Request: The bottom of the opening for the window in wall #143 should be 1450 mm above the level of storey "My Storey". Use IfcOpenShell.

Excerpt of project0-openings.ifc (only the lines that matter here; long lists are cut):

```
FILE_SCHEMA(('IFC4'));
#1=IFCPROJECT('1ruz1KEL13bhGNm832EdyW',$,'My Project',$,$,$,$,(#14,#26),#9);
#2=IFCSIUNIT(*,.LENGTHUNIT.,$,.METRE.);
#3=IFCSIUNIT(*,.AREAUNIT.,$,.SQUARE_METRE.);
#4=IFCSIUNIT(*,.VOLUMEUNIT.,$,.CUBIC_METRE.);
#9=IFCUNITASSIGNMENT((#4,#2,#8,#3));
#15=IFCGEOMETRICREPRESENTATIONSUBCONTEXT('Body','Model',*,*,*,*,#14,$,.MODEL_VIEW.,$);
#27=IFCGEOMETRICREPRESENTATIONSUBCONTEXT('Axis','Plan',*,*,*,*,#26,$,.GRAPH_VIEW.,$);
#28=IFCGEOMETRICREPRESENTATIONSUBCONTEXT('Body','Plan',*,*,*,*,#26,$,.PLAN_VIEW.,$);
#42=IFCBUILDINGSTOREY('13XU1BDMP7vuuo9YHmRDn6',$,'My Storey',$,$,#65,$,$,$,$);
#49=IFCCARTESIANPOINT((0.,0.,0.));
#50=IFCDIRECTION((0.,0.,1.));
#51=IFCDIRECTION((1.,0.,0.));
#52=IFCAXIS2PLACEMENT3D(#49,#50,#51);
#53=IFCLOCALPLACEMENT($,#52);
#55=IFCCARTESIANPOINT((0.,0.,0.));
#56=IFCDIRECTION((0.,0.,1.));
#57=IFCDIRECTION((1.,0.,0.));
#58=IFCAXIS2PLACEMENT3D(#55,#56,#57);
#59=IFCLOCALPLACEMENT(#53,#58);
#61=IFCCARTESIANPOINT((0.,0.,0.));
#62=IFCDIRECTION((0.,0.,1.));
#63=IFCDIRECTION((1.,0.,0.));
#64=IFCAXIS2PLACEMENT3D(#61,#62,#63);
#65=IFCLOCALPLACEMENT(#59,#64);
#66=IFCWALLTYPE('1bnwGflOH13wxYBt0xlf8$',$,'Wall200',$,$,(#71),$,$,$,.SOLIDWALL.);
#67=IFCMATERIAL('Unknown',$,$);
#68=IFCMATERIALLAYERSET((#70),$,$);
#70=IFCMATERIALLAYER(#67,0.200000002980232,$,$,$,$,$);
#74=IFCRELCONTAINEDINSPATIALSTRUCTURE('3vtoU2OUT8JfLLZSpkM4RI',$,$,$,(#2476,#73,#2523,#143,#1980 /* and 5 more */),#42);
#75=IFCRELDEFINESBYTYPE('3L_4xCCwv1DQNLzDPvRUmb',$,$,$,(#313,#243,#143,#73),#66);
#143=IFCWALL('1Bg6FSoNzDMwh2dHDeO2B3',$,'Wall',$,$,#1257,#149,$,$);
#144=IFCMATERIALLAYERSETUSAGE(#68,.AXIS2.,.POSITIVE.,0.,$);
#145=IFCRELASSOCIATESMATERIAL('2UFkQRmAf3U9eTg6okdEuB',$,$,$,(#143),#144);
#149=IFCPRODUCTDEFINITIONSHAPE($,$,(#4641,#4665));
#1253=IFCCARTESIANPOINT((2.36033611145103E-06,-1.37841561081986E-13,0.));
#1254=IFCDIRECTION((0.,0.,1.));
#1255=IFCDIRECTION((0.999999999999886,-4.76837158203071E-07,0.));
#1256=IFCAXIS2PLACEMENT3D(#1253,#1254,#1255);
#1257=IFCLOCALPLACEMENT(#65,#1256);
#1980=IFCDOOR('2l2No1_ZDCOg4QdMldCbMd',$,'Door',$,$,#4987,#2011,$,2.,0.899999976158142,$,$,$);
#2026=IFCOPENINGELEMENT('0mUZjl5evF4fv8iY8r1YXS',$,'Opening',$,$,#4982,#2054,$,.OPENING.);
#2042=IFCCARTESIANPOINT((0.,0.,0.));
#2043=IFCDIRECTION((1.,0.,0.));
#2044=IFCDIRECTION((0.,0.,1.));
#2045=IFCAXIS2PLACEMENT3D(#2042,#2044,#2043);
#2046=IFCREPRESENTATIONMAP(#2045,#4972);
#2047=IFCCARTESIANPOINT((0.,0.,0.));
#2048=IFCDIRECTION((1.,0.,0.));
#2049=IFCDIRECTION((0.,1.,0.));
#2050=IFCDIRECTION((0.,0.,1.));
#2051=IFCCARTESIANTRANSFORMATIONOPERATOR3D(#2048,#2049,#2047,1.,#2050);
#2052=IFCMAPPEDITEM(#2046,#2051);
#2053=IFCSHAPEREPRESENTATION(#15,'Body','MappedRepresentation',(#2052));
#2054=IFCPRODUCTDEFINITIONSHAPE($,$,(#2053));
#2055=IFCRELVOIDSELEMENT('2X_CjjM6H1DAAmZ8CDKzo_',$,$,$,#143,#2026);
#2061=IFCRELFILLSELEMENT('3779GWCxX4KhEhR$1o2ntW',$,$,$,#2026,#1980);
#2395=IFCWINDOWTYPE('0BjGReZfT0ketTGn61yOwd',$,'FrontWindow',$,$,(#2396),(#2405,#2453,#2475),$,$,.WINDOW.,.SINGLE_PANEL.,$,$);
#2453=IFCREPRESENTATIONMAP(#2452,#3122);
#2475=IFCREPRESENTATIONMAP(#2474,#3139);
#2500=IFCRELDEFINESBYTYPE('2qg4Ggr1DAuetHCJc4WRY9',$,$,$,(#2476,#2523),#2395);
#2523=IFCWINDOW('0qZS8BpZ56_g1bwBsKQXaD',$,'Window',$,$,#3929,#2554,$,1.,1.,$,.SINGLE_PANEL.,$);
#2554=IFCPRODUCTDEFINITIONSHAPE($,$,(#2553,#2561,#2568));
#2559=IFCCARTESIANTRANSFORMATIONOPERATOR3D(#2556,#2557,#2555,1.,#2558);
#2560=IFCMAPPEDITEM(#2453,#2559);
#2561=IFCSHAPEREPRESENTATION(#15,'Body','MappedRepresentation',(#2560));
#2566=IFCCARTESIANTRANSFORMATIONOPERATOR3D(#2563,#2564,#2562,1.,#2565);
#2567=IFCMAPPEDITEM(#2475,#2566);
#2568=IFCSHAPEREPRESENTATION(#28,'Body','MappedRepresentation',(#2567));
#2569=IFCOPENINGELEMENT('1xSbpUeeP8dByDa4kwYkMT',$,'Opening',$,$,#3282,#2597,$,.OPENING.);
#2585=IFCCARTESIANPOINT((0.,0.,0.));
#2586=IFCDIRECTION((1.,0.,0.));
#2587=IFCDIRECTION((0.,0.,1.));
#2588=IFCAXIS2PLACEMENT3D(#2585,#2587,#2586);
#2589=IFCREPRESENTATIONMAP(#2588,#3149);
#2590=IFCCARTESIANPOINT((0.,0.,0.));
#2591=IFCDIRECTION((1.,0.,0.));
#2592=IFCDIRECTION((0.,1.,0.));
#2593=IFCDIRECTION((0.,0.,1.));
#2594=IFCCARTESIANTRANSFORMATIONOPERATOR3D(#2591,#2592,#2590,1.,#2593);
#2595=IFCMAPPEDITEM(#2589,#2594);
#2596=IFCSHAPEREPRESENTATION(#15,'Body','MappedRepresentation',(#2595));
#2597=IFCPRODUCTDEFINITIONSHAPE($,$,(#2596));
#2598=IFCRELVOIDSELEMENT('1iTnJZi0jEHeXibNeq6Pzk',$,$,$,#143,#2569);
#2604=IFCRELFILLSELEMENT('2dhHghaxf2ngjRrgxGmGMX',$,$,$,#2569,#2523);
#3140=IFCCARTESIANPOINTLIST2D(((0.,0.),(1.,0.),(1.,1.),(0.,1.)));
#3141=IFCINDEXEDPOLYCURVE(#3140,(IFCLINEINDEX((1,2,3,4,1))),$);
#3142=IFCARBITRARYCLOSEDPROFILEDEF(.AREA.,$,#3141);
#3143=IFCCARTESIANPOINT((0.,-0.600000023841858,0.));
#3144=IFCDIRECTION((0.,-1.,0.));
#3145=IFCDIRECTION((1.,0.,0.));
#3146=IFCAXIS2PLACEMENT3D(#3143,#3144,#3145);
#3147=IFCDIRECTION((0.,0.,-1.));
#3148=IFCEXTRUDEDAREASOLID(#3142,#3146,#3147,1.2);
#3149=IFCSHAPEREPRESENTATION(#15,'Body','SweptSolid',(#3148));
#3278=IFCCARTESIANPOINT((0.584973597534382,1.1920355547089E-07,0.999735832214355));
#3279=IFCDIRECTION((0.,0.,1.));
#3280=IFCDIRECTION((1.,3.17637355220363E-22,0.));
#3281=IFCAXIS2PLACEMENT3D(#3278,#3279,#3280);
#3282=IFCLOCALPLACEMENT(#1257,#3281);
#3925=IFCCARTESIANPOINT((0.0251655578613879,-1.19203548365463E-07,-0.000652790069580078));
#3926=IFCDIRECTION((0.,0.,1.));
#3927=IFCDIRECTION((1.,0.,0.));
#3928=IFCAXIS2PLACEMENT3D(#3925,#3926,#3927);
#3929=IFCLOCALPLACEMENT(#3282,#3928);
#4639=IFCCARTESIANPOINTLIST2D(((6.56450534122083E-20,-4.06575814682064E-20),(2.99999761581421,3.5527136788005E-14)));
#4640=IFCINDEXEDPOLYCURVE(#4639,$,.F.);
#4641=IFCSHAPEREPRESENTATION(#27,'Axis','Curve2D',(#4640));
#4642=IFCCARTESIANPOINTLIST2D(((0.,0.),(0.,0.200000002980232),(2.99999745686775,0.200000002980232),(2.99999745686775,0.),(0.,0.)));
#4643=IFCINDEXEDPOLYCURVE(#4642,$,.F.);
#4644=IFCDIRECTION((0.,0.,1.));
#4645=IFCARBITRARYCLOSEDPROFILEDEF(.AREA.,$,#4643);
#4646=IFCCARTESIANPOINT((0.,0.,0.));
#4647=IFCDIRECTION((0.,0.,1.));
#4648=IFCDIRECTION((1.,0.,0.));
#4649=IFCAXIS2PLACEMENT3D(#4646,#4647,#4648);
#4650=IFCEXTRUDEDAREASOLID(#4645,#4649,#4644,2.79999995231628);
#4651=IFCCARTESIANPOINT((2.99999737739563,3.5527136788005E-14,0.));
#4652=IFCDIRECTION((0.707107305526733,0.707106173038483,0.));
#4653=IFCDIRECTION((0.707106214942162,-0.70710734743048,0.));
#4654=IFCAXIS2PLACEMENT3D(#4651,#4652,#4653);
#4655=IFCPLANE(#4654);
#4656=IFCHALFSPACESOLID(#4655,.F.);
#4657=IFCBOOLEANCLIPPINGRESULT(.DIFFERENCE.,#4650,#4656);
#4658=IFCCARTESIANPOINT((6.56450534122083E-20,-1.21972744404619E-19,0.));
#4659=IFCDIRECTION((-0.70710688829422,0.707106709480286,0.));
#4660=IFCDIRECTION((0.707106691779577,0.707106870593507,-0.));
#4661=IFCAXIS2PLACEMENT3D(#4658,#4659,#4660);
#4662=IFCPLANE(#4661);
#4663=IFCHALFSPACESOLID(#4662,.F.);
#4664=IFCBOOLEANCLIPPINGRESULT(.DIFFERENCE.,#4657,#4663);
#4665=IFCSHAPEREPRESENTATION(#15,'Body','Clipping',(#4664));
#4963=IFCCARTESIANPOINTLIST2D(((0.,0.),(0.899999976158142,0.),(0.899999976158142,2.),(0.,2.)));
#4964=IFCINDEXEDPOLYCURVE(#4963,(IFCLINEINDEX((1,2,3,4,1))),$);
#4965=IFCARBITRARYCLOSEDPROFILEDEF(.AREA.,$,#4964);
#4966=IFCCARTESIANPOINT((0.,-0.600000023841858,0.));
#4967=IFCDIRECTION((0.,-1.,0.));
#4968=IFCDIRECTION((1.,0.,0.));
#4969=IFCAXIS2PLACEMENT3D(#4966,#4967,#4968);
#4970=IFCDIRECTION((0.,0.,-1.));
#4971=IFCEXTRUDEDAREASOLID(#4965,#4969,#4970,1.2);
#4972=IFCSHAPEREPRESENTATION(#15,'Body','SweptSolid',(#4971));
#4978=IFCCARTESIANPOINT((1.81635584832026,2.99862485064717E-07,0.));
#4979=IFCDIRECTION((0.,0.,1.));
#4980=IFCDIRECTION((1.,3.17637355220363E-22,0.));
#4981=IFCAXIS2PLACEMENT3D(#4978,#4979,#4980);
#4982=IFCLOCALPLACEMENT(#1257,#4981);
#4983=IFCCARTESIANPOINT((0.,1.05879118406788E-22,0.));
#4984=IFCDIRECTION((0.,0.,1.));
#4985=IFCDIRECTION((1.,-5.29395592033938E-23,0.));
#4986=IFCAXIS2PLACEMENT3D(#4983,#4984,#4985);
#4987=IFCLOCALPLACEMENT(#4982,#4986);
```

```python
import numpy as np
import ifcopenshell
import ifcopenshell.api.geometry
import ifcopenshell.geom
import ifcopenshell.util.element
import ifcopenshell.util.placement
import ifcopenshell.util.shape
import ifcopenshell.util.unit

model = ifcopenshell.open("project0-openings.ifc")
unit_scale = ifcopenshell.util.unit.calculate_unit_scale(model)

window = model.by_id(2523)
opening = window.FillsVoids[0].RelatingOpeningElement
storey = ifcopenshell.util.element.get_container(window, ifc_class="IfcBuildingStorey")
level = ifcopenshell.util.placement.get_local_placement(storey.ObjectPlacement)[2, 3]

# The opening's origin need not be at the sill, so measure its lowest point.
shape = ifcopenshell.geom.create_shape(ifcopenshell.geom.settings(), opening)
bottom = ifcopenshell.util.shape.get_shape_bottom_elevation(shape, shape.geometry) / unit_scale
dz = level + 1.45 - bottom

shift = np.array([0.0, 0.0, dz])
# The window is placed relative to its opening, so it follows when the opening moves.
matrix = ifcopenshell.util.placement.get_local_placement(opening.ObjectPlacement)
matrix[:3, 3] += shift
ifcopenshell.api.geometry.edit_object_placement(
    model, product=opening, matrix=matrix, is_si=False, should_transform_children=True
)

print(f"moved by {dz * unit_scale:+.3f} m")

model.write("project0-openings_edited.ifc")
```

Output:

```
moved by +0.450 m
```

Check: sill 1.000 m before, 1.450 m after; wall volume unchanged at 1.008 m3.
